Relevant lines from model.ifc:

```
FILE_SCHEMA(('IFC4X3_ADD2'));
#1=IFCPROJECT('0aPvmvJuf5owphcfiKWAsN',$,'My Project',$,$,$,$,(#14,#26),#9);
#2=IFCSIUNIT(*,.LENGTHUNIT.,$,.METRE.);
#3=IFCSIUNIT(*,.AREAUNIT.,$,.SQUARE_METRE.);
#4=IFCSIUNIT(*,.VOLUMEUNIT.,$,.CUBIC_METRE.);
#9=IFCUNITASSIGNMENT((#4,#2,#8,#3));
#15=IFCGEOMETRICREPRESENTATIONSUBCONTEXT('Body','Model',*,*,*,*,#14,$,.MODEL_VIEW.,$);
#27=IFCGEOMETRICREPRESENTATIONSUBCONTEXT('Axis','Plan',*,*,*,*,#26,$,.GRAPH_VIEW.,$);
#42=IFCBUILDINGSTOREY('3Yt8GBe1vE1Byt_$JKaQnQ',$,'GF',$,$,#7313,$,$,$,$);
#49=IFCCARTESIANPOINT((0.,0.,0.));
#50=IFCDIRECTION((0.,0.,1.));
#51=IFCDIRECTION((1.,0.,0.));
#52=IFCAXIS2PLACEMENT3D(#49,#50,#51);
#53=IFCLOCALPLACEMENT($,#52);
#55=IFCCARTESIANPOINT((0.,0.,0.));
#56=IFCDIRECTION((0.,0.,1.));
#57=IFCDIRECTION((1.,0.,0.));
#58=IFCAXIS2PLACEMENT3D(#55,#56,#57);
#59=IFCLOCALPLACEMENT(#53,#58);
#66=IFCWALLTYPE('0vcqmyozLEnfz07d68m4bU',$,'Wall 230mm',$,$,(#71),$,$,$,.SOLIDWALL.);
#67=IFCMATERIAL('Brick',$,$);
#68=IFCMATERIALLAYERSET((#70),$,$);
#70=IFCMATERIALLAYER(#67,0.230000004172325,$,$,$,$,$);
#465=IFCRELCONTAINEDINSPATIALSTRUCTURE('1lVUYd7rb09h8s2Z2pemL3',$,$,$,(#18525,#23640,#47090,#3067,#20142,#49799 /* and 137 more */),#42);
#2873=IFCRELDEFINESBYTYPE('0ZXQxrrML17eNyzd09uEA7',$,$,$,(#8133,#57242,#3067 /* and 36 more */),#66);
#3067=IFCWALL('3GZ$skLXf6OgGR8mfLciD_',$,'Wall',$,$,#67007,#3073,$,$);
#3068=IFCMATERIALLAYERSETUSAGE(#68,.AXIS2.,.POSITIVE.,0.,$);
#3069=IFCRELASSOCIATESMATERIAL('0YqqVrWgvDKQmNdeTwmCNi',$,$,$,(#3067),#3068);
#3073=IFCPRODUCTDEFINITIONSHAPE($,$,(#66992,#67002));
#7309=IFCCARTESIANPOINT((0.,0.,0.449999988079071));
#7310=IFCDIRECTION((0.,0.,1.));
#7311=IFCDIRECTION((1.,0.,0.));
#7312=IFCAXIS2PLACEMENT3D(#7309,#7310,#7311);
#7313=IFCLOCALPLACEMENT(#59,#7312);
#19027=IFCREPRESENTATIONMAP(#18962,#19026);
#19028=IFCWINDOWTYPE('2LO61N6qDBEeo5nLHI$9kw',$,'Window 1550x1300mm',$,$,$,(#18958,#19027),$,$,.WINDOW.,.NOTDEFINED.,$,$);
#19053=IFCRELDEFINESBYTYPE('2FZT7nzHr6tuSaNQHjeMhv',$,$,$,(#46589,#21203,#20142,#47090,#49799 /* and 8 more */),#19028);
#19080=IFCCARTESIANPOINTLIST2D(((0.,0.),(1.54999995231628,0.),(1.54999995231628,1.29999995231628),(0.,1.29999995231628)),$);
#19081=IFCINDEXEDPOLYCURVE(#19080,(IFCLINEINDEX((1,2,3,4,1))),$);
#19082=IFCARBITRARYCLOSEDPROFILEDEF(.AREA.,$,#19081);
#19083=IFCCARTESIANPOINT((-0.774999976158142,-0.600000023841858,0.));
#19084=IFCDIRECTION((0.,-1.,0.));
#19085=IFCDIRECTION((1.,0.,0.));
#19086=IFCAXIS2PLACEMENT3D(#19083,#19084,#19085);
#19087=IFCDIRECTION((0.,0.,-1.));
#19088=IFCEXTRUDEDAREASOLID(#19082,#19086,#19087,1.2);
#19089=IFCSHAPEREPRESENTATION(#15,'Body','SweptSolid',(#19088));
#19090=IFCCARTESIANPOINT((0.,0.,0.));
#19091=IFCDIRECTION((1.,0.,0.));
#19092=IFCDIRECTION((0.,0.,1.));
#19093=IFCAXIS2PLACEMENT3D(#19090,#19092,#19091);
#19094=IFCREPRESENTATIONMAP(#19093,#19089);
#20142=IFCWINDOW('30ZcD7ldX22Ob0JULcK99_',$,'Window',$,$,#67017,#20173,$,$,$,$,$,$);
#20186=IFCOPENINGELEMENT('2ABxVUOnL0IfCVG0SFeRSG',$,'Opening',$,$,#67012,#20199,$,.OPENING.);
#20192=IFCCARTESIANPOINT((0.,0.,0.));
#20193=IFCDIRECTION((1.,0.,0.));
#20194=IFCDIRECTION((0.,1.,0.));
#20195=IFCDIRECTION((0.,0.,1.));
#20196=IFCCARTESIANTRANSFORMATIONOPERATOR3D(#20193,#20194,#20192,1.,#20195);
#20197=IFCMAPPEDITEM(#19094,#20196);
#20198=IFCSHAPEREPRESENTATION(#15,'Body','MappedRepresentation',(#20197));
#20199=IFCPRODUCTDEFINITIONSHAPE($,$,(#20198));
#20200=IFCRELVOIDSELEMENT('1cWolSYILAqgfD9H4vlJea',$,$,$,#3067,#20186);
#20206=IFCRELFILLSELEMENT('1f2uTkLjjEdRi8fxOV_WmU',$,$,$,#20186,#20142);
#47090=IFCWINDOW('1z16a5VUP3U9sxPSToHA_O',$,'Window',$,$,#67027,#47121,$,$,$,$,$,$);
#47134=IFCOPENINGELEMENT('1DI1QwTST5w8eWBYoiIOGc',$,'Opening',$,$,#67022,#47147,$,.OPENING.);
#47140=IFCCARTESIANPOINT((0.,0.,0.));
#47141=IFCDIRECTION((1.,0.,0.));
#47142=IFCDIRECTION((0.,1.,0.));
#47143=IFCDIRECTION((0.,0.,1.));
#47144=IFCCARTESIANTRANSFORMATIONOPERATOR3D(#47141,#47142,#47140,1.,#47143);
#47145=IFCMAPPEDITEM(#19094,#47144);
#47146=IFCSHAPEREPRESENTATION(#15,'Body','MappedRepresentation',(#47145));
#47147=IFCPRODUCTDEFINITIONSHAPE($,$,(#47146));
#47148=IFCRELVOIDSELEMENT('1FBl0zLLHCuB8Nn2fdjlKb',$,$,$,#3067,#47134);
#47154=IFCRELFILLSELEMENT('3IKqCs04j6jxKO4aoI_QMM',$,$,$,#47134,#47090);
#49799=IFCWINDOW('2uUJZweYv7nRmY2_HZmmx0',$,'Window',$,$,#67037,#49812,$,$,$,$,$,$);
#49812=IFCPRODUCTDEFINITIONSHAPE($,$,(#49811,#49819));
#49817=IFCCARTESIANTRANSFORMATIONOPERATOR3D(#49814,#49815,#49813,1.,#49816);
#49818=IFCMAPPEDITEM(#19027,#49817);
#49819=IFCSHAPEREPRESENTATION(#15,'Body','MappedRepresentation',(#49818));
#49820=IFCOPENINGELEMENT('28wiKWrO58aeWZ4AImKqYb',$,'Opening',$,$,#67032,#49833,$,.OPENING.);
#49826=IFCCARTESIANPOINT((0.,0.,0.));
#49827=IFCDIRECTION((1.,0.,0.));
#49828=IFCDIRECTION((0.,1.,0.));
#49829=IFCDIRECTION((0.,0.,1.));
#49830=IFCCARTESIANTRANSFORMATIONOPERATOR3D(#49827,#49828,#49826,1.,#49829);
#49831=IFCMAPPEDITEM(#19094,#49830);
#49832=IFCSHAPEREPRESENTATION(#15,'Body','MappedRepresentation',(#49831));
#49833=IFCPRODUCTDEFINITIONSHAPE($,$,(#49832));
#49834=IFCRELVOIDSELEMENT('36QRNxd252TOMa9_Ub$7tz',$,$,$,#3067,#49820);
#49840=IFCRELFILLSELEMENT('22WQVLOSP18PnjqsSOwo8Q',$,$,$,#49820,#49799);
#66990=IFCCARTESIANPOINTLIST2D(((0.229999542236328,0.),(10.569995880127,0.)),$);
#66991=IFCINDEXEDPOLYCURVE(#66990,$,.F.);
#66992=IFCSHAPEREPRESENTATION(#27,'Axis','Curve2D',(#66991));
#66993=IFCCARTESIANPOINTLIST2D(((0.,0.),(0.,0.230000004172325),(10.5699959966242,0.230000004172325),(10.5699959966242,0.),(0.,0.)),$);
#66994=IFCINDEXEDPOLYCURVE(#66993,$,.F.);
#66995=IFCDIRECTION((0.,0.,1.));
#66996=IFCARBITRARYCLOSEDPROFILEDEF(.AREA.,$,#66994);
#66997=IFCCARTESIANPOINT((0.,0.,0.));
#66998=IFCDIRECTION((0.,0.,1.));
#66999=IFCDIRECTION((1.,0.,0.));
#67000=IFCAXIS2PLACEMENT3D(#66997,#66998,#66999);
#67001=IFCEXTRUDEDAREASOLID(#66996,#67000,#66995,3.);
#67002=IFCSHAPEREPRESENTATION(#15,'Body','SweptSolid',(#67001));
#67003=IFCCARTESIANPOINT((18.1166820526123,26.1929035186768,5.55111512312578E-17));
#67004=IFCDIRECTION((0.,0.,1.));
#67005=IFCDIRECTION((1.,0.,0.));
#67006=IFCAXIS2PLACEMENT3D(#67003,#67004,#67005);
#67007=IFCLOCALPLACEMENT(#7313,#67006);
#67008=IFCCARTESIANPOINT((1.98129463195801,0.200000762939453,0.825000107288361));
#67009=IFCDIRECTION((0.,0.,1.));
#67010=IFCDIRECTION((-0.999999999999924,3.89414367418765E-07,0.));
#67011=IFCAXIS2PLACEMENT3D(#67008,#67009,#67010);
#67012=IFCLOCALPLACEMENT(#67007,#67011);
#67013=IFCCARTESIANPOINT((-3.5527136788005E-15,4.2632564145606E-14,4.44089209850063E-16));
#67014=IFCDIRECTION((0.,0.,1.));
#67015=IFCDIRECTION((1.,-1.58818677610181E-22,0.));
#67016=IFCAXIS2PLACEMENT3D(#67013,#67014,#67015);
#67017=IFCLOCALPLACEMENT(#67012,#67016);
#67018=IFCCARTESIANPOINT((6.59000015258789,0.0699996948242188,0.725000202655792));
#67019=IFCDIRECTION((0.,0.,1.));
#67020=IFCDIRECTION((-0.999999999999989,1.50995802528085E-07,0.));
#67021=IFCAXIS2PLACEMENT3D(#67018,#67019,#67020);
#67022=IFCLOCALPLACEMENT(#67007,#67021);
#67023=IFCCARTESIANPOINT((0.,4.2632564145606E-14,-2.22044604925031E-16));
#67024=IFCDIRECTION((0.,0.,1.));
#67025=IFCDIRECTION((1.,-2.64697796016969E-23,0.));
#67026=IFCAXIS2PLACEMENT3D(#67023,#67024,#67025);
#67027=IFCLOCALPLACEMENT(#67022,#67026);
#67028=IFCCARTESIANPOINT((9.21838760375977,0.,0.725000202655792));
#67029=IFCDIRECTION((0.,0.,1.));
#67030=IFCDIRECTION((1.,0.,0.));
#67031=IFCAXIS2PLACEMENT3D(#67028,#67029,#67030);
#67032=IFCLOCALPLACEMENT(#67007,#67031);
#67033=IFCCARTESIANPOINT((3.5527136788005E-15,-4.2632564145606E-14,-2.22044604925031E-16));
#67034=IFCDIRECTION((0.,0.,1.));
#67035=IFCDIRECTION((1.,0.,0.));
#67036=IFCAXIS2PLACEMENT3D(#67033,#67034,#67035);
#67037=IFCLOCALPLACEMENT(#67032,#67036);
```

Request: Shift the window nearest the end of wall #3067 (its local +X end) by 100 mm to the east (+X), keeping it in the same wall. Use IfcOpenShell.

```python
import ifcopenshell
import ifcopenshell.api.geometry
import ifcopenshell.util.placement

model = ifcopenshell.open("model.ifc")

window = model.by_id(49799)
opening = window.FillsVoids[0].RelatingOpeningElement
wall = opening.VoidsElements[0].RelatingBuildingElement

wall_matrix = ifcopenshell.util.placement.get_local_placement(wall.ObjectPlacement)
shift = wall_matrix[:3, 0] * 0.1
before = ifcopenshell.util.placement.get_local_placement(window.ObjectPlacement)[:3, 3].copy()

# The window is placed relative to its opening, so it follows when the opening moves.
matrix = ifcopenshell.util.placement.get_local_placement(opening.ObjectPlacement)
matrix[:3, 3] += shift
ifcopenshell.api.geometry.edit_object_placement(
    model, product=opening, matrix=matrix, is_si=False, should_transform_children=True
)

after = ifcopenshell.util.placement.get_local_placement(window.ObjectPlacement)[:3, 3]
print("window moved by", (after - before).round(3) + 0.0)

model.write("model_updated.ifc")
```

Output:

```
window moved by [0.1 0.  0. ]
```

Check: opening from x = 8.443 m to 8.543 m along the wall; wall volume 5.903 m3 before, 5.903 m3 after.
